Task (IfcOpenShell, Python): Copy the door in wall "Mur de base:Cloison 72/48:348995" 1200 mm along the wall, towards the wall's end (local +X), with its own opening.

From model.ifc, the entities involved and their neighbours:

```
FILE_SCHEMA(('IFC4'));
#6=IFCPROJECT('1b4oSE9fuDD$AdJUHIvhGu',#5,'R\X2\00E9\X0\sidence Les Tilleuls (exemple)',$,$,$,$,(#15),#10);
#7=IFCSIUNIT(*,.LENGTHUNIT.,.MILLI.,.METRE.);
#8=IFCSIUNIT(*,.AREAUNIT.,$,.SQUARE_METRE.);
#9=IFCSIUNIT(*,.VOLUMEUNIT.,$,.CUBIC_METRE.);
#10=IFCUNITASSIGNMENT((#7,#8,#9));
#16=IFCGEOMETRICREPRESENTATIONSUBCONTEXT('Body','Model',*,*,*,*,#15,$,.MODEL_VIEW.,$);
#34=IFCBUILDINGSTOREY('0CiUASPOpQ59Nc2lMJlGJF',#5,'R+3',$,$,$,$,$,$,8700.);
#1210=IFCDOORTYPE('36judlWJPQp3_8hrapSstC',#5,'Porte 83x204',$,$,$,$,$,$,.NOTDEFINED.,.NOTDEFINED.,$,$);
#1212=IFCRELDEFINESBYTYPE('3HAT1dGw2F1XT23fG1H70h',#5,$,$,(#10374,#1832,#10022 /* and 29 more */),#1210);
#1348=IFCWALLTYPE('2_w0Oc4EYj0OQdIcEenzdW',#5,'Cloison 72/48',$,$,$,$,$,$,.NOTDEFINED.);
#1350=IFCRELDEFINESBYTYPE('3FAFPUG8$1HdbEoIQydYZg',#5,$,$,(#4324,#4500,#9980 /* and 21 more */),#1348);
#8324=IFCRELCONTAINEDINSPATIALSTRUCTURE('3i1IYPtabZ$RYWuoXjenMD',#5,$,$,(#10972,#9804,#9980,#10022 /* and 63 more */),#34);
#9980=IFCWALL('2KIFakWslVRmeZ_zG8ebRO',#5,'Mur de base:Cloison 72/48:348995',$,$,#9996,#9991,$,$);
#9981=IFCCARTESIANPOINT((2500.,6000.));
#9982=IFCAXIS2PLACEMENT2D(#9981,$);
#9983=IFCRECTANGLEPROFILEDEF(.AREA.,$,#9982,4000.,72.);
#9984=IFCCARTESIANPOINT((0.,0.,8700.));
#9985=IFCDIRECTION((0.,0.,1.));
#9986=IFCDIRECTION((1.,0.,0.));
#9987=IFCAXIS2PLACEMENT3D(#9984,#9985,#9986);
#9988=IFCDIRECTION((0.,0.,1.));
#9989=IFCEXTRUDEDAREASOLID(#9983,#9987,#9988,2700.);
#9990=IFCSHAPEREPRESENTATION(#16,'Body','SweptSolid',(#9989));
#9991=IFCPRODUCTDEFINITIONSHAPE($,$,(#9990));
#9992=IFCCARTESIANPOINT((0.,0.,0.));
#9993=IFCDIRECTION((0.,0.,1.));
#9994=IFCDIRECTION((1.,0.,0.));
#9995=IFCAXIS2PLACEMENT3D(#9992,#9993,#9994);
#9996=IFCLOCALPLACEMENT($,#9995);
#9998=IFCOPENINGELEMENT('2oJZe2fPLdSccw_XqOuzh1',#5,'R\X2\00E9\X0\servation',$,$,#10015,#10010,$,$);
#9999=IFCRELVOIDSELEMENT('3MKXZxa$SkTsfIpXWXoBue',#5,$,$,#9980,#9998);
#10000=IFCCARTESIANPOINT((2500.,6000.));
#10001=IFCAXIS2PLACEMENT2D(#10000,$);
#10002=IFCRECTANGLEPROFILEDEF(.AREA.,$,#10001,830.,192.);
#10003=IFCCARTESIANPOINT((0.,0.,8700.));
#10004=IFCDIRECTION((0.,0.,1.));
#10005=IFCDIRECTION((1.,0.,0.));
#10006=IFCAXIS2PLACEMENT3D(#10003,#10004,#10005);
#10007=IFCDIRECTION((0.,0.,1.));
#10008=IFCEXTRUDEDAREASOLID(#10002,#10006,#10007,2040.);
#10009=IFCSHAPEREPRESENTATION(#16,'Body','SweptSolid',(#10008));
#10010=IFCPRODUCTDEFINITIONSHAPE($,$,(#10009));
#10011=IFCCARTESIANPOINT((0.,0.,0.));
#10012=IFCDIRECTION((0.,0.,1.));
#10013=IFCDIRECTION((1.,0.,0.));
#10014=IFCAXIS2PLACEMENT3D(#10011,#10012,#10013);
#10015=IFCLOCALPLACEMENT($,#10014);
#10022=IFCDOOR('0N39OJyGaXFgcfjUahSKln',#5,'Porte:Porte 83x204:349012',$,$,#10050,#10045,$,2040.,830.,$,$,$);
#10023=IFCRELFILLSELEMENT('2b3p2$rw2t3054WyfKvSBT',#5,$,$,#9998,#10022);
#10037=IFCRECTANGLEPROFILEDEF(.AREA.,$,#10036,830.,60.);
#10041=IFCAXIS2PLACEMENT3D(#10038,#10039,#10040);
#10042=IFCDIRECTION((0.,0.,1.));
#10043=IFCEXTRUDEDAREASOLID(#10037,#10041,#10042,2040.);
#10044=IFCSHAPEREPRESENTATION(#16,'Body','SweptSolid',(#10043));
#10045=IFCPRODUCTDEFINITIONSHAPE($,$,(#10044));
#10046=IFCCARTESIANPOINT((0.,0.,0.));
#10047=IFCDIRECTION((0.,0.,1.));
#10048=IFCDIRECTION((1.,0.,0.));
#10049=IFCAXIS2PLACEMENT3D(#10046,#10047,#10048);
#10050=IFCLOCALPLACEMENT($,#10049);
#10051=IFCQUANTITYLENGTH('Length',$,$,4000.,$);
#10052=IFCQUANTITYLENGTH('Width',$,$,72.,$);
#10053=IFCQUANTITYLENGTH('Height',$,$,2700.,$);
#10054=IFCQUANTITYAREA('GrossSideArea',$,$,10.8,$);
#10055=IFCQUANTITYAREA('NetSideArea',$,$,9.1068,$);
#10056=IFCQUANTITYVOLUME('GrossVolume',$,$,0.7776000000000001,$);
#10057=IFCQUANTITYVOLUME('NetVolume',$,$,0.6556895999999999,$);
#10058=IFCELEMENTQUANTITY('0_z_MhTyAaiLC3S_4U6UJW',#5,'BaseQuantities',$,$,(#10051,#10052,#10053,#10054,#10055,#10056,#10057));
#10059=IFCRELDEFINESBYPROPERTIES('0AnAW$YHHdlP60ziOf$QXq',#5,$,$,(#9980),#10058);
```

```python
import ifcopenshell
import ifcopenshell.api.feature
import ifcopenshell.api.geometry
import ifcopenshell.api.pset
import ifcopenshell.api.root
import ifcopenshell.geom
import ifcopenshell.util.element
import ifcopenshell.util.placement
import ifcopenshell.util.shape
import ifcopenshell.util.unit

model = ifcopenshell.open("model.ifc")
unit_scale = ifcopenshell.util.unit.calculate_unit_scale(model)
area_scale = ifcopenshell.util.unit.calculate_unit_scale(model, "AREAUNIT")
volume_scale = ifcopenshell.util.unit.calculate_unit_scale(model, "VOLUMEUNIT")
settings = ifcopenshell.geom.settings()


def volume(element):
    """Net volume in cubic metres, openings subtracted."""
    shape = ifcopenshell.geom.create_shape(settings, element)
    return ifcopenshell.util.shape.get_volume(shape.geometry)


def reuse_history(source, copy):
    """copy_class also copies each property set's owner history, people and application; keep the originals."""
    for rel in copy.IsDefinedBy:
        if rel.is_a("IfcRelDefinesByProperties") and (history := rel.RelatingPropertyDefinition.OwnerHistory):
            rel.RelatingPropertyDefinition.OwnerHistory = source.OwnerHistory
            ifcopenshell.util.element.remove_deep2(model, history)


door = model.by_guid("0N39OJyGaXFgcfjUahSKln")
opening = door.FillsVoids[0].RelatingOpeningElement
wall = opening.VoidsElements[0].RelatingBuildingElement
before = volume(wall)
shift = ifcopenshell.util.placement.get_local_placement(wall.ObjectPlacement)[:3, 0] * 1.2 / unit_scale

# copy_class copies the void relationship, type, container and properties, but no geometry.
new_opening = ifcopenshell.api.root.copy_class(model, product=opening)
new_opening.Representation = ifcopenshell.util.element.copy_deep(
    model, opening.Representation, exclude=["IfcGeometricRepresentationContext", "IfcRepresentationMap"]
)
reuse_history(opening, new_opening)
new_door = ifcopenshell.api.root.copy_class(model, product=door)
new_door.Representation = ifcopenshell.util.element.copy_deep(
    model, door.Representation, exclude=["IfcGeometricRepresentationContext", "IfcRepresentationMap"]
)
new_door.Name = "Porte:Porte 83x204"
reuse_history(door, new_door)
ifcopenshell.api.feature.add_filling(model, opening=new_opening, element=new_door)

for old, new in ((opening, new_opening), (door, new_door)):
    matrix = ifcopenshell.util.placement.get_local_placement(old.ObjectPlacement)
    matrix[:3, 3] += shift
    ifcopenshell.api.geometry.edit_object_placement(model, product=new, matrix=matrix, is_si=False)

after = volume(wall)
thickness = 0.072  # wall thickness in metres

# Update the wall's stored quantities.
qto = model.by_id(ifcopenshell.util.element.get_pset(wall, "BaseQuantities", should_inherit=False)["id"])
ifcopenshell.api.pset.edit_qto(model, qto=qto, properties={
    "NetSideArea": after / thickness / area_scale,
    "NetVolume": after / volume_scale,
})

print(f"wall volume {before:.3f} -> {after:.3f} m3")

model.write("model_v2.ifc")
```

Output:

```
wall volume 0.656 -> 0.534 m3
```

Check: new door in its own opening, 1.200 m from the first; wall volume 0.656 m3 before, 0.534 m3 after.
